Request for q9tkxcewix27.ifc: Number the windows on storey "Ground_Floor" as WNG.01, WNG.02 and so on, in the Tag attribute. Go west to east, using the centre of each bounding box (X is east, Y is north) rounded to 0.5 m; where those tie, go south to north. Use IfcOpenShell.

First a look at what the model holds.

```python
import ifcopenshell
import ifcopenshell.util.element
import ifcopenshell.util.placement

model = ifcopenshell.open("q9tkxcewix27.ifc")
print(model.schema)
storey = next(s for s in model.by_type("IfcBuildingStorey") if s.Name == "Ground_Floor")
windows = [e for e in ifcopenshell.util.element.get_decomposition(storey) if e.is_a("IfcWindow")]
for e in sorted(windows, key=lambda e: e.id()):
    origin = ifcopenshell.util.placement.get_local_placement(e.ObjectPlacement)[:3, 3]
    print(e.id(), e.Tag, e.Name, origin.round(2) + 0.0, sep=" | ")
```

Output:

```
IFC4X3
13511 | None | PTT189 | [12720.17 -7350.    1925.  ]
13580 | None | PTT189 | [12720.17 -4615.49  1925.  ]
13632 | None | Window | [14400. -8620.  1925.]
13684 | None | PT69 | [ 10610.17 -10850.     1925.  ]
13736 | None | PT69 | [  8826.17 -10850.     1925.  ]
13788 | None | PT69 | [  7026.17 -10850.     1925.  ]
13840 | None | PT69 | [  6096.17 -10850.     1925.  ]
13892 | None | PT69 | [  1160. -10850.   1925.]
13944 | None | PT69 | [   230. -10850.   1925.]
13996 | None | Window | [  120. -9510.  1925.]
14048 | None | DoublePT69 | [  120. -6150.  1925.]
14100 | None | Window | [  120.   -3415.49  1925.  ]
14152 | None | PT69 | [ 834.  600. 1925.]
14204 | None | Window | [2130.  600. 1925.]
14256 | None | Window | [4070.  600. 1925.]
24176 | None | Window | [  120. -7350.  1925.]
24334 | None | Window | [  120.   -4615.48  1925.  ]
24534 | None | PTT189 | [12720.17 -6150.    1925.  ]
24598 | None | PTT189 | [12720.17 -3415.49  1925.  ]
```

```python
import ifcopenshell
import ifcopenshell.geom
import ifcopenshell.util.element
import ifcopenshell.util.shape

model = ifcopenshell.open("q9tkxcewix27.ifc")
settings = ifcopenshell.geom.settings()
settings.set("use-world-coords", True)


def centre(element):
    shape = ifcopenshell.geom.create_shape(settings, element)
    return ifcopenshell.util.shape.get_bbox_centroid(shape.geometry)


storey = next(s for s in model.by_type("IfcBuildingStorey") if s.Name == "Ground_Floor")
windows = [e for e in ifcopenshell.util.element.get_decomposition(storey) if e.is_a("IfcWindow")]

# Insertion points can sit at a corner or the storey origin, so sort by the geometry (in metres).
centres = {e: centre(e) for e in windows}
windows.sort(key=lambda e: (round(centres[e][0] / 0.5), centres[e][1]))

for i, e in enumerate(windows, start=1):
    number = f"WNG.{i:02d}"
    e.Tag = number
    print(e.id(), number)

model.write("q9tkxcewix27_updated.ifc")
```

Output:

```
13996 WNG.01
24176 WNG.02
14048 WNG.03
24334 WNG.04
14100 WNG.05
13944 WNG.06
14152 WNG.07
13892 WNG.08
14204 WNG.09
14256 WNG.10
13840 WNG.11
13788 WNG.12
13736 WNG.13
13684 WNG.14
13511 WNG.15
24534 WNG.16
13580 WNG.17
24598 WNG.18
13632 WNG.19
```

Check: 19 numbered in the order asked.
